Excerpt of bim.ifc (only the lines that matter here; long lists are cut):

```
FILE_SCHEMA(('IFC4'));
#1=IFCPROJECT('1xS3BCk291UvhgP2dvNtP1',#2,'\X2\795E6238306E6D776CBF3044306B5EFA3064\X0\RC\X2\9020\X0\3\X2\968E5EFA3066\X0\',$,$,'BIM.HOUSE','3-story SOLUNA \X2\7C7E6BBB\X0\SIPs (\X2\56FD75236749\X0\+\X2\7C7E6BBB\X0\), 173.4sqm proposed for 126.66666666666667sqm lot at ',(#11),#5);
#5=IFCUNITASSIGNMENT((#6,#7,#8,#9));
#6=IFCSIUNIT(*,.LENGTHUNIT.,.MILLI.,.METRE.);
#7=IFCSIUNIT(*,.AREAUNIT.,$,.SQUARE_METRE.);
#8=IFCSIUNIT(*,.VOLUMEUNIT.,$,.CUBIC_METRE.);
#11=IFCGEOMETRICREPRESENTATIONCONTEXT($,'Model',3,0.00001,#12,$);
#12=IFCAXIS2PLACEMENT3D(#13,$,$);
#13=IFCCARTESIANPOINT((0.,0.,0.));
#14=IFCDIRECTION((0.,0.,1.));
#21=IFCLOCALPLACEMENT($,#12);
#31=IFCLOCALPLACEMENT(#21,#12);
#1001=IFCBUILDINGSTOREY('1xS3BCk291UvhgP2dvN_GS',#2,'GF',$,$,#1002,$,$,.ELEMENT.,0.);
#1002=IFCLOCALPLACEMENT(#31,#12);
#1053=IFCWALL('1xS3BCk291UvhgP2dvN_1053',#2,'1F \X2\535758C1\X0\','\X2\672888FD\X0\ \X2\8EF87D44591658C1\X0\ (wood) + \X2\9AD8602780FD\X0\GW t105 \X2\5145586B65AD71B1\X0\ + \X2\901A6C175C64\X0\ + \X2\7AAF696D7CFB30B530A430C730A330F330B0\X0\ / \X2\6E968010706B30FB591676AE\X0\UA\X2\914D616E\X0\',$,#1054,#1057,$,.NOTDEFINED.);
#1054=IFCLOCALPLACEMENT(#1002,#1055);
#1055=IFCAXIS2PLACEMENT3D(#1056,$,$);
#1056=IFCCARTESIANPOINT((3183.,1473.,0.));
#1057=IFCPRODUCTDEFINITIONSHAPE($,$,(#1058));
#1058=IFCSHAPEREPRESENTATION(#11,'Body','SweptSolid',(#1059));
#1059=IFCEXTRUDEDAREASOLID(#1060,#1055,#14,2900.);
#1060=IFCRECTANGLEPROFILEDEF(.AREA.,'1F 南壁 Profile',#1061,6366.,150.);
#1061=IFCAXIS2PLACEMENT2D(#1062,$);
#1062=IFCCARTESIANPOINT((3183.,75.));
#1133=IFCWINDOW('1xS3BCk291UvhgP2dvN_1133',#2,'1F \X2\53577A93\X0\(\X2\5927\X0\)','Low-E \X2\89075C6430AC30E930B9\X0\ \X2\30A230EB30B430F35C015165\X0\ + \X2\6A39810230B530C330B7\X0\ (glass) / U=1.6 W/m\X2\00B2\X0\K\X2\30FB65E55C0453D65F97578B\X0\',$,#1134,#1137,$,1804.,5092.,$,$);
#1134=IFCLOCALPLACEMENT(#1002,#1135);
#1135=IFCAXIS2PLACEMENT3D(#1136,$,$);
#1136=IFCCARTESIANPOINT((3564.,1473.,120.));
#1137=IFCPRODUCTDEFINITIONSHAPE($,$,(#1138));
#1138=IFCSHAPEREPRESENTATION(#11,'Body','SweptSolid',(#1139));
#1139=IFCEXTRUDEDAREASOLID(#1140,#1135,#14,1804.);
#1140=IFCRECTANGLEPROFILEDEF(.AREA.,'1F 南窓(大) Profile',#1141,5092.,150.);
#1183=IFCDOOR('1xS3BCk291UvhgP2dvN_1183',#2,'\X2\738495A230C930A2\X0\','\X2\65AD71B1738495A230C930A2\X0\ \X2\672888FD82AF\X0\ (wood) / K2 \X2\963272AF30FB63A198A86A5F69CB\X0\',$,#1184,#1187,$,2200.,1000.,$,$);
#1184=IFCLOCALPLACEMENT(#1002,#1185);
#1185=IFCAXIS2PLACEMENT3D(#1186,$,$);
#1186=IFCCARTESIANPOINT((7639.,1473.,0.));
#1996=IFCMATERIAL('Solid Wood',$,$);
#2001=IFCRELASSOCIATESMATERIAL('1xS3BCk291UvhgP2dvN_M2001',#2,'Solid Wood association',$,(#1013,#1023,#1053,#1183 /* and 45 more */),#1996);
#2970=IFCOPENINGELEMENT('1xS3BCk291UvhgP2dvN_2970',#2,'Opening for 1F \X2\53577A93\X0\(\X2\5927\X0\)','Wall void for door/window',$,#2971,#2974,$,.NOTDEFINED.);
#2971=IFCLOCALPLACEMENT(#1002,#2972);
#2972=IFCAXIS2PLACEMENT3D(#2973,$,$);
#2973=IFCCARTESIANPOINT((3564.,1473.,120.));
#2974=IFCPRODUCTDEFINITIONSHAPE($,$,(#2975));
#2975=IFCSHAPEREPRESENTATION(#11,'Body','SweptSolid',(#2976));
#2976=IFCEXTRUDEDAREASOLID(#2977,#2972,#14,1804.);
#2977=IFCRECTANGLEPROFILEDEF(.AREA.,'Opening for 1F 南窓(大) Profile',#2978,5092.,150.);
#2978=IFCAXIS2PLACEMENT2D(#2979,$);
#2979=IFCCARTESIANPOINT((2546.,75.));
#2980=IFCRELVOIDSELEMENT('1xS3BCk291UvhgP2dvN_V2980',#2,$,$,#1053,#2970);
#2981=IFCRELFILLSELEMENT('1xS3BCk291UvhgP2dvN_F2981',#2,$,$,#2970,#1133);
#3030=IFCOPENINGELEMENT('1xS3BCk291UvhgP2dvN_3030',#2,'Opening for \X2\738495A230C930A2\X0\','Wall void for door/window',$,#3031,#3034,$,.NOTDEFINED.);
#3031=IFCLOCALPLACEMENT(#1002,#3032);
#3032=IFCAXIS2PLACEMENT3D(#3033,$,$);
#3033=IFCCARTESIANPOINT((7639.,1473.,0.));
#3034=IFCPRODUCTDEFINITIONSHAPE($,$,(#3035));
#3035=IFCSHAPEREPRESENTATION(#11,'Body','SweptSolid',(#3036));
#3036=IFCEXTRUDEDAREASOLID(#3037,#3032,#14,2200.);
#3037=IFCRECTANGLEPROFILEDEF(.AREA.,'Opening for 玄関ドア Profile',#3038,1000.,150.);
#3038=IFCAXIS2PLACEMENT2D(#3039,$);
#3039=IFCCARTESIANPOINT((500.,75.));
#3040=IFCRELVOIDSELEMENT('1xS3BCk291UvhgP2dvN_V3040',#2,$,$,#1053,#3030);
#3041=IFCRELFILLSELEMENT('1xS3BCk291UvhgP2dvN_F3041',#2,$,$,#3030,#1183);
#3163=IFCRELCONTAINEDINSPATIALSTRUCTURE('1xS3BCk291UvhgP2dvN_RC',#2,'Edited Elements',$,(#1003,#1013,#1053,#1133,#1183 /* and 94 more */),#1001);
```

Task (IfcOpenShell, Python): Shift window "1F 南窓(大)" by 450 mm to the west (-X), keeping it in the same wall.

```python
import ifcopenshell
import ifcopenshell.api.geometry
import ifcopenshell.util.placement

model = ifcopenshell.open("bim.ifc")

window = model.by_guid("1xS3BCk291UvhgP2dvN_1133")
opening = window.FillsVoids[0].RelatingOpeningElement
wall = opening.VoidsElements[0].RelatingBuildingElement

wall_matrix = ifcopenshell.util.placement.get_local_placement(wall.ObjectPlacement)
shift = wall_matrix[:3, 0] * -450.0
before = ifcopenshell.util.placement.get_local_placement(window.ObjectPlacement)[:3, 3].copy()

# The window is not placed relative to its opening, so move both.
for product in (opening, window):
    matrix = ifcopenshell.util.placement.get_local_placement(product.ObjectPlacement)
    matrix[:3, 3] += shift
    ifcopenshell.api.geometry.edit_object_placement(model, product=product, matrix=matrix, is_si=False)

after = ifcopenshell.util.placement.get_local_placement(window.ObjectPlacement)[:3, 3]
print("window moved by", (after - before).round(3) + 0.0)

model.write("bim_edited.ifc")
```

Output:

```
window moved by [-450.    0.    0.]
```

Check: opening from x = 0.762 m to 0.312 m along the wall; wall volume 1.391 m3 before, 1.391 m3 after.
